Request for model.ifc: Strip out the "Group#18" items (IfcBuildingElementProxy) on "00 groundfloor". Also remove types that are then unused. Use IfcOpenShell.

First a look at what the model holds.

```python
import ifcopenshell
import ifcopenshell.util.element

model = ifcopenshell.open("model.ifc")
print(model.schema)
storey = next(s for s in model.by_type("IfcBuildingStorey") if s.Name == "00 groundfloor")
proxies = [e for e in ifcopenshell.util.element.get_decomposition(storey) if e.is_a("IfcBuildingElementProxy")]
seen = {}
for e in proxies:
    element_type = ifcopenshell.util.element.get_type(e)
    name = element_type.Name if element_type not in (None, e) else None
    seen[name] = seen.get(name, 0) + 1
for name, count in sorted(seen.items(), key=str):
    print(count, "x", name)
```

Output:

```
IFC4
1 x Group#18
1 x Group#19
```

```python
import ifcopenshell
import ifcopenshell.api.root
import ifcopenshell.util.element

model = ifcopenshell.open("model.ifc")

storey = next(s for s in model.by_type("IfcBuildingStorey") if s.Name == "00 groundfloor")
proxies = [e for e in ifcopenshell.util.element.get_decomposition(storey) if e.is_a("IfcBuildingElementProxy")]
targets = [e for e in proxies if (t := ifcopenshell.util.element.get_type(e)) not in (None, e) and t.Name == "Group#18"]
types = {ifcopenshell.util.element.get_type(e) for e in targets} - {None, *targets}

for e in targets:
    ifcopenshell.api.root.remove_product(model, product=e)
print(len(targets), "removed")

unused = [t for t in types if not ifcopenshell.util.element.get_types(t)]
for t in unused:
    ifcopenshell.api.root.remove_product(model, product=t)
print(len(unused), "unused types removed")

model.write("model_edited.ifc")
```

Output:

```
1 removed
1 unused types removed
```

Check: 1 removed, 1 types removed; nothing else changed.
